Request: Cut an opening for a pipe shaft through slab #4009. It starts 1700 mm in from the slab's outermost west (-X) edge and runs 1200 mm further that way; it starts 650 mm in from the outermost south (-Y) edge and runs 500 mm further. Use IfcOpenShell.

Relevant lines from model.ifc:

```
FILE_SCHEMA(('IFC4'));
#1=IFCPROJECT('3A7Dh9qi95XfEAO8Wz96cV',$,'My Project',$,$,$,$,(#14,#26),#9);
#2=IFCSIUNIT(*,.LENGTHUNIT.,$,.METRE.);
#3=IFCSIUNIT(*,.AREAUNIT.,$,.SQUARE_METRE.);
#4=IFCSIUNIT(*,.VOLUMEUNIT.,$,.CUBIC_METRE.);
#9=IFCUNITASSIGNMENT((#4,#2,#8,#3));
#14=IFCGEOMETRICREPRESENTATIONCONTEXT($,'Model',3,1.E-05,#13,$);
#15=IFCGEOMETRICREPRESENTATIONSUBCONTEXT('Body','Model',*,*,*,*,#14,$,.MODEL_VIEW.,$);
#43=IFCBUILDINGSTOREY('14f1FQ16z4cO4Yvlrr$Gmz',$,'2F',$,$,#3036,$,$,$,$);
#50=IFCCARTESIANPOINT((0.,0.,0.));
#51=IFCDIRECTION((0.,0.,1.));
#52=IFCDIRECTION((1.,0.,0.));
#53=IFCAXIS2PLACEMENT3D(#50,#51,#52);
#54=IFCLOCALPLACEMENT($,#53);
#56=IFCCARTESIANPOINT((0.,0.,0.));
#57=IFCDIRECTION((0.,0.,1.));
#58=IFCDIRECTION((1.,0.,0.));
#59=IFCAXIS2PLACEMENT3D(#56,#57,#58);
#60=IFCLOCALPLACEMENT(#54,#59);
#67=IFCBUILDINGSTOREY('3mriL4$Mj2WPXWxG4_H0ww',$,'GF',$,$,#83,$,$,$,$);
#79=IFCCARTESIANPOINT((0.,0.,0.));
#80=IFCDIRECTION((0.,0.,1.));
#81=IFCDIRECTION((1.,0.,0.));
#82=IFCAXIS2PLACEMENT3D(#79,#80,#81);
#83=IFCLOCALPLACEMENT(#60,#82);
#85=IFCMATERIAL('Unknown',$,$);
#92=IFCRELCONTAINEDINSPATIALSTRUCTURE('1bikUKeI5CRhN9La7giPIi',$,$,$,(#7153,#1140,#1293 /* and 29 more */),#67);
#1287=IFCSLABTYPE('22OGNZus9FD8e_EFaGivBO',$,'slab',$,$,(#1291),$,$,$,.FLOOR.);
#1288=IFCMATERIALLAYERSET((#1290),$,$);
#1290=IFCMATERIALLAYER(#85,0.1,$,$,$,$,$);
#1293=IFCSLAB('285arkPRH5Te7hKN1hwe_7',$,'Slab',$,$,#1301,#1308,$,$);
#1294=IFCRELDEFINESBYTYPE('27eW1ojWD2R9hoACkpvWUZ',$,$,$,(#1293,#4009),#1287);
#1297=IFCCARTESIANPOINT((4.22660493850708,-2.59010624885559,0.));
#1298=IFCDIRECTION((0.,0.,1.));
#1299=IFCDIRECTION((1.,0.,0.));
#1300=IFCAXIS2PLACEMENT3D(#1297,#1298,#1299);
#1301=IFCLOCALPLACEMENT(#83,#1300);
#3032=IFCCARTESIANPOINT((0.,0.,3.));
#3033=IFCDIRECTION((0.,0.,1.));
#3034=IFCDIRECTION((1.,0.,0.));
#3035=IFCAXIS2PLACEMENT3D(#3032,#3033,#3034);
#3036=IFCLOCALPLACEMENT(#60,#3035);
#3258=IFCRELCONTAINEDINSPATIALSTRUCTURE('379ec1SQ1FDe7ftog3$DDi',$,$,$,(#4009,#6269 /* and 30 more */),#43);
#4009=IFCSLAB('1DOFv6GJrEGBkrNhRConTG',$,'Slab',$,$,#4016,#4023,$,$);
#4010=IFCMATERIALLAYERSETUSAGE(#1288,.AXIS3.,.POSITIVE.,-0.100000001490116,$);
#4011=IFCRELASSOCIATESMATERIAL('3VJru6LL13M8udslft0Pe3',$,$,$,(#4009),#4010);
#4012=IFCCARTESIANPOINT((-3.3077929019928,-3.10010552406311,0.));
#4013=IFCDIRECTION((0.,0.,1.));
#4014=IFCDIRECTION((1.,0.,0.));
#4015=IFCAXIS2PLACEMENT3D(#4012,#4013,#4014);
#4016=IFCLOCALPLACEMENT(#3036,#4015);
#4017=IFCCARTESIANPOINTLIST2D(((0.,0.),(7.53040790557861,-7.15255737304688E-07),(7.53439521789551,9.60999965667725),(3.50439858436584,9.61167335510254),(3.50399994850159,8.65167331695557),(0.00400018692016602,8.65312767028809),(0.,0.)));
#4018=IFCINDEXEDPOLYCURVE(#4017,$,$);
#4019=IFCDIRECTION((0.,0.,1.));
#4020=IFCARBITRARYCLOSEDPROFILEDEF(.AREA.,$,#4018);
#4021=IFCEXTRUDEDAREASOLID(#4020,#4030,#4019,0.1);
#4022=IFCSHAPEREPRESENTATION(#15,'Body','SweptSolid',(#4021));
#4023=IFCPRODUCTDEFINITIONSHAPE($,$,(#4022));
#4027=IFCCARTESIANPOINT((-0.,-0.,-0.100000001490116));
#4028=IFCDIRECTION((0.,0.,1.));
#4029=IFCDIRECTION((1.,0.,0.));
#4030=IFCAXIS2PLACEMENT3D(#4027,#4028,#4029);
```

```python
import numpy as np
import ifcopenshell
import ifcopenshell.api.feature
import ifcopenshell.api.geometry
import ifcopenshell.api.root
import ifcopenshell.geom
import ifcopenshell.util.placement
import ifcopenshell.util.representation
import ifcopenshell.util.shape
import ifcopenshell.util.unit

model = ifcopenshell.open("model.ifc")
unit_scale = ifcopenshell.util.unit.calculate_unit_scale(model)
settings = ifcopenshell.geom.settings()


def volume(element):
    """Net volume in cubic metres, openings subtracted."""
    shape = ifcopenshell.geom.create_shape(settings, element)
    return ifcopenshell.util.shape.get_volume(shape.geometry)


slab = model.by_guid("1DOFv6GJrEGBkrNhRConTG")
before = volume(slab)

# Extent in the slab's own axes, in metres. The edges named are its -X and -Y sides.
slab_shape = ifcopenshell.geom.create_shape(settings, slab)
vertices = ifcopenshell.util.shape.get_vertices(slab_shape.geometry)
x_min, y_min, bottom = vertices.min(axis=0)
top = vertices[:, 2].max()

opening = ifcopenshell.api.root.create_entity(model, ifc_class="IfcOpeningElement", name="Pipe shaft opening", predefined_type="OPENING")
context = ifcopenshell.util.representation.get_context(model, "Model", "Body", "MODEL_VIEW")
width, depth = 1.2, 0.5
outline = [(0.0, 0.0), (width, 0.0), (width, depth), (0.0, depth), (0.0, 0.0)]
# Overshoot both faces by 50 mm so the cut is clean.
shape = ifcopenshell.api.geometry.add_slab_representation(
    model, context=context, depth=top - bottom + 0.1, polyline=outline
)
ifcopenshell.api.geometry.assign_representation(model, product=opening, representation=shape)

matrix = ifcopenshell.util.placement.get_local_placement(slab.ObjectPlacement)
matrix[:, 3] = matrix @ np.append(np.array([x_min + 1.7, y_min + 0.65, bottom - 0.05]) / unit_scale, 1.0)
ifcopenshell.api.geometry.edit_object_placement(model, product=opening, matrix=matrix, is_si=False)
ifcopenshell.api.feature.add_feature(model, feature=opening, element=slab)

after = volume(slab)

print(f"slab volume {before:.3f} -> {after:.3f} m3")

model.write("model_v2.ifc")
```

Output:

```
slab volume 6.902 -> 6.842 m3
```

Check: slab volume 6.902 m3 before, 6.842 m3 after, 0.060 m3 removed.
